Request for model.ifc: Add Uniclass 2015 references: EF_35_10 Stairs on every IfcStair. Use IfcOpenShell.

First a look at what the model holds.

```python
import ifcopenshell

model = ifcopenshell.open("model.ifc")
print(model.schema)
print("classifications:", [c.Name for c in model.by_type("IfcClassification")])
for ifc_class in ("IfcDoor", "IfcRoof", "IfcStair", "IfcWall", "IfcWindow"):
    print(ifc_class, len(model.by_type(ifc_class)))
```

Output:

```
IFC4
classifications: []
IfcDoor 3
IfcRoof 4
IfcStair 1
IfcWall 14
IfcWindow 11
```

```python
import ifcopenshell
import ifcopenshell.api.classification

model = ifcopenshell.open("model.ifc")

system = ifcopenshell.api.classification.add_classification(model, classification="Uniclass 2015")

codes = {
    "IfcStair": ("EF_35_10", "Stairs"),
}
for ifc_class, (code, name) in codes.items():
    products = model.by_type(ifc_class)
    ifcopenshell.api.classification.add_reference(
        model, products=products, classification=system, identification=code, name=name
    )
    print(code, len(products))

model.write("model_v2.ifc")
```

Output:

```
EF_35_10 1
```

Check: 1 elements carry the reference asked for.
